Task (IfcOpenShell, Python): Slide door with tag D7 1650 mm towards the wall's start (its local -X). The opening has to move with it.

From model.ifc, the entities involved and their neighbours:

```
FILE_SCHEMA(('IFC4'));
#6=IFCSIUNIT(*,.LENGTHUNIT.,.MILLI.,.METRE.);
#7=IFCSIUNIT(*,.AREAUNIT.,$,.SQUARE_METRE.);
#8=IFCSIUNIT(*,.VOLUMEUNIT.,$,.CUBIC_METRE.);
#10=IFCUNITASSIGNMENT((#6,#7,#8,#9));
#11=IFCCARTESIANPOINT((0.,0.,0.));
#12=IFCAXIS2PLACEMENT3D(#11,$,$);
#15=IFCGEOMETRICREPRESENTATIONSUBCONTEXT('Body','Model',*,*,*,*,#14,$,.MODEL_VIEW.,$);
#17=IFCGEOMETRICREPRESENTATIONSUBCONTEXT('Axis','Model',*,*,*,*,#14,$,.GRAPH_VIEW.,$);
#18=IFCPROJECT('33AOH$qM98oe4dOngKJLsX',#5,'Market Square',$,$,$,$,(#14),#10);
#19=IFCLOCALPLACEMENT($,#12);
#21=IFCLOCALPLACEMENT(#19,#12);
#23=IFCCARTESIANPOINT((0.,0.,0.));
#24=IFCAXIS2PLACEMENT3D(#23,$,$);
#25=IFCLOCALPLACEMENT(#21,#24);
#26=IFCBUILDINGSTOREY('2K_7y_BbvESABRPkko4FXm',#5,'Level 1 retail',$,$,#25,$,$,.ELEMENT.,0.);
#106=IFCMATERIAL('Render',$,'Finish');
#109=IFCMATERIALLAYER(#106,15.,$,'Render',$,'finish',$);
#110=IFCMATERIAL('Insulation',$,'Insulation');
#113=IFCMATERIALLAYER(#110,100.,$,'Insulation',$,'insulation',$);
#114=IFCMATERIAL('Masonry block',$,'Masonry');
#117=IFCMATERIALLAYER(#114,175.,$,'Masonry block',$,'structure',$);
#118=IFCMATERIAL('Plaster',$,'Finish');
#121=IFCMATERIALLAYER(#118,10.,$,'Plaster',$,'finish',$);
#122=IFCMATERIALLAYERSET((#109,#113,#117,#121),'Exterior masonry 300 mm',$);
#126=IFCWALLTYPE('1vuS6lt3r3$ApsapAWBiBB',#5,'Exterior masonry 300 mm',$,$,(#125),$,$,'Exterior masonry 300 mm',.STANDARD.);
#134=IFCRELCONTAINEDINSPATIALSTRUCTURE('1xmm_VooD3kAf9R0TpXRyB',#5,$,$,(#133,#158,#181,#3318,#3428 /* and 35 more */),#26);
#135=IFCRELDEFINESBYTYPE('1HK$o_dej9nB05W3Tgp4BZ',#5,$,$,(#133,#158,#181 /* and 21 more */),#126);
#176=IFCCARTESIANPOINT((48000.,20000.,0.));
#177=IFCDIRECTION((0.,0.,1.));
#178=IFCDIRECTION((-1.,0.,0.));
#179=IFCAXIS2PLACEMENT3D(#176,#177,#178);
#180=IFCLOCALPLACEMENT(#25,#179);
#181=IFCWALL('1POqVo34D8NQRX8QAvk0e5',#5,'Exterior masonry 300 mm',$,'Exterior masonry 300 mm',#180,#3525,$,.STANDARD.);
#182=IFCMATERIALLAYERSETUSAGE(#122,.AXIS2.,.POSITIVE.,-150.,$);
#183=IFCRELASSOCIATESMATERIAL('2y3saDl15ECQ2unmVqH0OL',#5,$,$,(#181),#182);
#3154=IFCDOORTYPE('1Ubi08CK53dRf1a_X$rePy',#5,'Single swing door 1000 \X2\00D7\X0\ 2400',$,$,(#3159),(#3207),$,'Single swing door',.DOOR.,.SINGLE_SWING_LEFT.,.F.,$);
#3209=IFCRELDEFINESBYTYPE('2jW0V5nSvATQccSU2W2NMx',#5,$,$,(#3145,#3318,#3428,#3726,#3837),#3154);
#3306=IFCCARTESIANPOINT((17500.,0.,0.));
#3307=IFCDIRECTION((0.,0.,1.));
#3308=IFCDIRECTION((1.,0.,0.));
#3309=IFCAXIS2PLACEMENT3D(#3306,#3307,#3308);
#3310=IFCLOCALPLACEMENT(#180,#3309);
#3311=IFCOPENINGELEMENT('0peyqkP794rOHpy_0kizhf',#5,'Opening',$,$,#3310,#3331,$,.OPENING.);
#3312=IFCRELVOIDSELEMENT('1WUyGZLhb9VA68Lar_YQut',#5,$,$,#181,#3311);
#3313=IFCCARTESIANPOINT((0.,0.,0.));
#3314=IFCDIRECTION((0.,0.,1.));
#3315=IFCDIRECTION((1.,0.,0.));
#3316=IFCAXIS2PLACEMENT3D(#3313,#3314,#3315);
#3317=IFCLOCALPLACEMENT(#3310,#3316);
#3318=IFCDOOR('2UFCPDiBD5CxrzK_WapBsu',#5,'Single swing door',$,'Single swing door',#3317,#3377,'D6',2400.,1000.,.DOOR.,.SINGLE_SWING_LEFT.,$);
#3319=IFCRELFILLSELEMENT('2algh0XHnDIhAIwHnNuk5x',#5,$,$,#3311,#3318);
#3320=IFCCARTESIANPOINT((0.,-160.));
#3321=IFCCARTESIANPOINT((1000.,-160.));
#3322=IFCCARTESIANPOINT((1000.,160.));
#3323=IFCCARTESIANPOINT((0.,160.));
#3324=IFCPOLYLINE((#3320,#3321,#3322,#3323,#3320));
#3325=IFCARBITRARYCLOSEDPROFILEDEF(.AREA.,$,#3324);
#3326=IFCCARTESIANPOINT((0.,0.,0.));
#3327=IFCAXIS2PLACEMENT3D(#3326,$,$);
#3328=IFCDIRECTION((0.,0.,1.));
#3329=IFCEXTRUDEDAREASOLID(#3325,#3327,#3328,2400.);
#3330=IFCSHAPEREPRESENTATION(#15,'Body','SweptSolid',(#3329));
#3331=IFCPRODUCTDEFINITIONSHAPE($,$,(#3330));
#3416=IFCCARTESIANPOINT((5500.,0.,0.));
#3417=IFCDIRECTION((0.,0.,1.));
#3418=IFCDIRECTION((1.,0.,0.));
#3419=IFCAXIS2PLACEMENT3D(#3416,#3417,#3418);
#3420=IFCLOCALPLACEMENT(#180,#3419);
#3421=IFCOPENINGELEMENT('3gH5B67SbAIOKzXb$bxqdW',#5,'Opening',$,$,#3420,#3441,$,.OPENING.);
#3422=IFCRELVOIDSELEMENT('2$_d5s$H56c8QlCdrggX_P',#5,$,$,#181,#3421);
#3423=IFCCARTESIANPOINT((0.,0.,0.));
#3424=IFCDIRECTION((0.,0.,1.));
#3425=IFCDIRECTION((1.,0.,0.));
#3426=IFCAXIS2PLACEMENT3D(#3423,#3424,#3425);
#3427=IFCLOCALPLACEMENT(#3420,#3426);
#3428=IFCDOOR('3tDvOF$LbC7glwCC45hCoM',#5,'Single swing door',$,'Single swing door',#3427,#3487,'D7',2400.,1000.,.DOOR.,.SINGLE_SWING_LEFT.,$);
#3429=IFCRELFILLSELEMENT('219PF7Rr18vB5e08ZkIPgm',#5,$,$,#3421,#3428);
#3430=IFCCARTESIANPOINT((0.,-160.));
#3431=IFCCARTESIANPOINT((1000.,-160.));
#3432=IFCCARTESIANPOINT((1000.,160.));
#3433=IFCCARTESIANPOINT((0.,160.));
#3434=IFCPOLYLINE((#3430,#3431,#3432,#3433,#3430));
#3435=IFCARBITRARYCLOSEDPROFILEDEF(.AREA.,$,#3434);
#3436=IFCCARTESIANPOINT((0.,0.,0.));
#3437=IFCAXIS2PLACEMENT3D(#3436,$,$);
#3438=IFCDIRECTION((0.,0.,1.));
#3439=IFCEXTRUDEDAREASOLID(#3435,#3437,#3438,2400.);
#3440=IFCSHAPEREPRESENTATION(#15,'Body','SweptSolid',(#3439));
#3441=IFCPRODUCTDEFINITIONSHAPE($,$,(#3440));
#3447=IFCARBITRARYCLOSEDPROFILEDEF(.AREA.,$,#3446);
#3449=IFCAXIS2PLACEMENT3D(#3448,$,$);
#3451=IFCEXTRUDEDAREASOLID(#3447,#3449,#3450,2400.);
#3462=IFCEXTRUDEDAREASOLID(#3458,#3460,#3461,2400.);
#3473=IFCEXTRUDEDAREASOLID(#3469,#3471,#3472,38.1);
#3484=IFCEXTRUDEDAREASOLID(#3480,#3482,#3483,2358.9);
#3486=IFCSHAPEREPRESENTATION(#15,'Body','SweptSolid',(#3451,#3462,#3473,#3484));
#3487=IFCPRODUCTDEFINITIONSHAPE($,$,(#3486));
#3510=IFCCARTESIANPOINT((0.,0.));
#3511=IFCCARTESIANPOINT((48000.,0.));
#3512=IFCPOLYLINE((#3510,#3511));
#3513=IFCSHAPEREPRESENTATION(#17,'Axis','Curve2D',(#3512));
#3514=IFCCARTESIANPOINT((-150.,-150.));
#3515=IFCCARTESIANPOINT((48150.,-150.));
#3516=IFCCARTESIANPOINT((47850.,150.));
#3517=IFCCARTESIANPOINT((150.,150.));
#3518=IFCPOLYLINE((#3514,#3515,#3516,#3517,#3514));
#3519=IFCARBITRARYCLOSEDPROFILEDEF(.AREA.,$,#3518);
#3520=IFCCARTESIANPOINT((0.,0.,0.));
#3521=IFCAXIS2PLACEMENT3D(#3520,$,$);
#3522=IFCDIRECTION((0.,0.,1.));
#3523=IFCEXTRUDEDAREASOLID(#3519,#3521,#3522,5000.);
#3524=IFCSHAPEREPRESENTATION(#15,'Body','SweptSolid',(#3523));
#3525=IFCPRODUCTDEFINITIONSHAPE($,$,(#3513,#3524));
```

```python
import ifcopenshell
import ifcopenshell.api.geometry
import ifcopenshell.util.placement
import ifcopenshell.util.unit

model = ifcopenshell.open("model.ifc")
unit_scale = ifcopenshell.util.unit.calculate_unit_scale(model)

door = model.by_guid("3tDvOF$LbC7glwCC45hCoM")
opening = door.FillsVoids[0].RelatingOpeningElement
wall = opening.VoidsElements[0].RelatingBuildingElement

wall_matrix = ifcopenshell.util.placement.get_local_placement(wall.ObjectPlacement)
shift = wall_matrix[:3, 0] * -1.65 / unit_scale
before = ifcopenshell.util.placement.get_local_placement(door.ObjectPlacement)[:3, 3].copy()

# The door is placed relative to its opening, so it follows when the opening moves.
matrix = ifcopenshell.util.placement.get_local_placement(opening.ObjectPlacement)
matrix[:3, 3] += shift
ifcopenshell.api.geometry.edit_object_placement(
    model, product=opening, matrix=matrix, is_si=False, should_transform_children=True
)

after = ifcopenshell.util.placement.get_local_placement(door.ObjectPlacement)[:3, 3]
print("door moved by", (after - before).round(3) + 0.0)

model.write("model_v2.ifc")
```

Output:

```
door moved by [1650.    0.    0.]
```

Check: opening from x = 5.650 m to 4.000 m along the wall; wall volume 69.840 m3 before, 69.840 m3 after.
